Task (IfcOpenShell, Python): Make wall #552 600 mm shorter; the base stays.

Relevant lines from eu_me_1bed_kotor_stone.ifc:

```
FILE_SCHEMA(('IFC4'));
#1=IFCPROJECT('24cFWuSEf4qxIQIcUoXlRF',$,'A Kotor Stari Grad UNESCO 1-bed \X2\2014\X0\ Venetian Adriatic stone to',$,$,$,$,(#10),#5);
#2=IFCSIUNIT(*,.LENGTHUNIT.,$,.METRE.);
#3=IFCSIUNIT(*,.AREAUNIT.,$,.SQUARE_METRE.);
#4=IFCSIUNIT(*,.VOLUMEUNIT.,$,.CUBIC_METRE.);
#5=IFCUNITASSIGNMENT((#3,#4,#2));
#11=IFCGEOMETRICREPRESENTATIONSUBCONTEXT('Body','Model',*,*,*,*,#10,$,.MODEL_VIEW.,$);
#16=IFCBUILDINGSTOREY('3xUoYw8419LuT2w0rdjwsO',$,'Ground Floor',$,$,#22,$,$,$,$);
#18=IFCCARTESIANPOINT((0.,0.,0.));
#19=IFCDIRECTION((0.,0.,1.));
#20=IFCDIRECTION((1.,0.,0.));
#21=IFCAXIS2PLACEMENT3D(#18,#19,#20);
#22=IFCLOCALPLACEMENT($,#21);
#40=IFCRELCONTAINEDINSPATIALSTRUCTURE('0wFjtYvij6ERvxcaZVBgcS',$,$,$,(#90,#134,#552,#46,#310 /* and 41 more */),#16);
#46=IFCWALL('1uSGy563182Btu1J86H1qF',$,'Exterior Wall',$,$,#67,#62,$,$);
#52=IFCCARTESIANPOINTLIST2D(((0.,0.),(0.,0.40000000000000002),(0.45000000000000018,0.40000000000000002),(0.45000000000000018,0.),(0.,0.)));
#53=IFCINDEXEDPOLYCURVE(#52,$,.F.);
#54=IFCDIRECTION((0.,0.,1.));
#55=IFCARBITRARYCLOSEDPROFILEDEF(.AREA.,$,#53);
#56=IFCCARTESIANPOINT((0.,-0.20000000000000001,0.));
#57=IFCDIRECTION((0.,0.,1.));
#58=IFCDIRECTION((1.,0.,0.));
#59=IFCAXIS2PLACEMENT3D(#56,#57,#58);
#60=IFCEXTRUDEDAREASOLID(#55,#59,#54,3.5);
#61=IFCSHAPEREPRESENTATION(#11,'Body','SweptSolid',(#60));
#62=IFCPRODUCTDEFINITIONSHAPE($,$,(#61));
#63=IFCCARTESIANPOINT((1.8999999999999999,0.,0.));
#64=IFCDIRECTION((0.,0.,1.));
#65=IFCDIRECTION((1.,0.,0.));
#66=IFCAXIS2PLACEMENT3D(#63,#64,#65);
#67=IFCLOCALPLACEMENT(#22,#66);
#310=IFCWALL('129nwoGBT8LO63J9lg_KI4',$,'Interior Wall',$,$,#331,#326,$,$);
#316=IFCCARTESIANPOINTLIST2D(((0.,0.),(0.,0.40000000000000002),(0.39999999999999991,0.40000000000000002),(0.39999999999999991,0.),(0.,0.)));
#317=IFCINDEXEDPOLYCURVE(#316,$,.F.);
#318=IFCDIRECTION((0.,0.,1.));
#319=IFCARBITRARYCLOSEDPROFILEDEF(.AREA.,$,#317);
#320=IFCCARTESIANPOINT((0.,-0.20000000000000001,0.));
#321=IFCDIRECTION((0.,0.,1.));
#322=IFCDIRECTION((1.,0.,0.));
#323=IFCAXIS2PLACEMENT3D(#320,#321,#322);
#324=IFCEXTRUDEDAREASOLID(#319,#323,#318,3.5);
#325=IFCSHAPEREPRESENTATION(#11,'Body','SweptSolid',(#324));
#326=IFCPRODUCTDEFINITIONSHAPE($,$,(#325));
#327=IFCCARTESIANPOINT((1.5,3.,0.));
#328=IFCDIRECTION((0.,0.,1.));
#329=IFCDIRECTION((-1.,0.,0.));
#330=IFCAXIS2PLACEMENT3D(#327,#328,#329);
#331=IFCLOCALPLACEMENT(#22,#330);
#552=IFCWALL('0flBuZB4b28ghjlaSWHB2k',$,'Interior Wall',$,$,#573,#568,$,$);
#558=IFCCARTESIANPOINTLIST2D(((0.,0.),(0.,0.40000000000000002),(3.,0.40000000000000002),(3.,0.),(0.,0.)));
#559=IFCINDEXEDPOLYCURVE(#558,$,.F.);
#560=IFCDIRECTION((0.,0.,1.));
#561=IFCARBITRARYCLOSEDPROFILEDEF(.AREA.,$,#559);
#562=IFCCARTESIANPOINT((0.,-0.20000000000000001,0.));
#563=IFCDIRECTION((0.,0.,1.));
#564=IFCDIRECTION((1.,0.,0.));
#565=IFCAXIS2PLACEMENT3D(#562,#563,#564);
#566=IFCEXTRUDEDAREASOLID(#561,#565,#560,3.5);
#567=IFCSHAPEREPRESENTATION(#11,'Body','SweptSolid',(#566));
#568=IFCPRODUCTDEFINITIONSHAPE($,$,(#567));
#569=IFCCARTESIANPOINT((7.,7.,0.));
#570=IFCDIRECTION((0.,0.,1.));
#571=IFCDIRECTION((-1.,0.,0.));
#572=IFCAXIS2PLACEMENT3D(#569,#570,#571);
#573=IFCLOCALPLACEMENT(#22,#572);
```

```python
import ifcopenshell
import ifcopenshell.geom
import ifcopenshell.util.representation
import ifcopenshell.util.shape

model = ifcopenshell.open("eu_me_1bed_kotor_stone.ifc")
settings = ifcopenshell.geom.settings()


def volume(element):
    """Net volume in cubic metres, openings subtracted."""
    shape = ifcopenshell.geom.create_shape(settings, element)
    return ifcopenshell.util.shape.get_volume(shape.geometry)


wall = model.by_id(552)
before = volume(wall)

body = ifcopenshell.util.representation.get_representation(wall, "Model", "Body")
solid = body.Items[0]
old_height = solid.Depth
solid.Depth -= 0.6
after = volume(wall)

print(f"height {old_height:g} -> {solid.Depth:g}, volume {before:.3f} -> {after:.3f} m3")

model.write("eu_me_1bed_kotor_stone_rev.ifc")
```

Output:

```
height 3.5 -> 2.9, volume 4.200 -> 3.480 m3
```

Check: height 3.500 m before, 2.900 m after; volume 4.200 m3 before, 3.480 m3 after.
